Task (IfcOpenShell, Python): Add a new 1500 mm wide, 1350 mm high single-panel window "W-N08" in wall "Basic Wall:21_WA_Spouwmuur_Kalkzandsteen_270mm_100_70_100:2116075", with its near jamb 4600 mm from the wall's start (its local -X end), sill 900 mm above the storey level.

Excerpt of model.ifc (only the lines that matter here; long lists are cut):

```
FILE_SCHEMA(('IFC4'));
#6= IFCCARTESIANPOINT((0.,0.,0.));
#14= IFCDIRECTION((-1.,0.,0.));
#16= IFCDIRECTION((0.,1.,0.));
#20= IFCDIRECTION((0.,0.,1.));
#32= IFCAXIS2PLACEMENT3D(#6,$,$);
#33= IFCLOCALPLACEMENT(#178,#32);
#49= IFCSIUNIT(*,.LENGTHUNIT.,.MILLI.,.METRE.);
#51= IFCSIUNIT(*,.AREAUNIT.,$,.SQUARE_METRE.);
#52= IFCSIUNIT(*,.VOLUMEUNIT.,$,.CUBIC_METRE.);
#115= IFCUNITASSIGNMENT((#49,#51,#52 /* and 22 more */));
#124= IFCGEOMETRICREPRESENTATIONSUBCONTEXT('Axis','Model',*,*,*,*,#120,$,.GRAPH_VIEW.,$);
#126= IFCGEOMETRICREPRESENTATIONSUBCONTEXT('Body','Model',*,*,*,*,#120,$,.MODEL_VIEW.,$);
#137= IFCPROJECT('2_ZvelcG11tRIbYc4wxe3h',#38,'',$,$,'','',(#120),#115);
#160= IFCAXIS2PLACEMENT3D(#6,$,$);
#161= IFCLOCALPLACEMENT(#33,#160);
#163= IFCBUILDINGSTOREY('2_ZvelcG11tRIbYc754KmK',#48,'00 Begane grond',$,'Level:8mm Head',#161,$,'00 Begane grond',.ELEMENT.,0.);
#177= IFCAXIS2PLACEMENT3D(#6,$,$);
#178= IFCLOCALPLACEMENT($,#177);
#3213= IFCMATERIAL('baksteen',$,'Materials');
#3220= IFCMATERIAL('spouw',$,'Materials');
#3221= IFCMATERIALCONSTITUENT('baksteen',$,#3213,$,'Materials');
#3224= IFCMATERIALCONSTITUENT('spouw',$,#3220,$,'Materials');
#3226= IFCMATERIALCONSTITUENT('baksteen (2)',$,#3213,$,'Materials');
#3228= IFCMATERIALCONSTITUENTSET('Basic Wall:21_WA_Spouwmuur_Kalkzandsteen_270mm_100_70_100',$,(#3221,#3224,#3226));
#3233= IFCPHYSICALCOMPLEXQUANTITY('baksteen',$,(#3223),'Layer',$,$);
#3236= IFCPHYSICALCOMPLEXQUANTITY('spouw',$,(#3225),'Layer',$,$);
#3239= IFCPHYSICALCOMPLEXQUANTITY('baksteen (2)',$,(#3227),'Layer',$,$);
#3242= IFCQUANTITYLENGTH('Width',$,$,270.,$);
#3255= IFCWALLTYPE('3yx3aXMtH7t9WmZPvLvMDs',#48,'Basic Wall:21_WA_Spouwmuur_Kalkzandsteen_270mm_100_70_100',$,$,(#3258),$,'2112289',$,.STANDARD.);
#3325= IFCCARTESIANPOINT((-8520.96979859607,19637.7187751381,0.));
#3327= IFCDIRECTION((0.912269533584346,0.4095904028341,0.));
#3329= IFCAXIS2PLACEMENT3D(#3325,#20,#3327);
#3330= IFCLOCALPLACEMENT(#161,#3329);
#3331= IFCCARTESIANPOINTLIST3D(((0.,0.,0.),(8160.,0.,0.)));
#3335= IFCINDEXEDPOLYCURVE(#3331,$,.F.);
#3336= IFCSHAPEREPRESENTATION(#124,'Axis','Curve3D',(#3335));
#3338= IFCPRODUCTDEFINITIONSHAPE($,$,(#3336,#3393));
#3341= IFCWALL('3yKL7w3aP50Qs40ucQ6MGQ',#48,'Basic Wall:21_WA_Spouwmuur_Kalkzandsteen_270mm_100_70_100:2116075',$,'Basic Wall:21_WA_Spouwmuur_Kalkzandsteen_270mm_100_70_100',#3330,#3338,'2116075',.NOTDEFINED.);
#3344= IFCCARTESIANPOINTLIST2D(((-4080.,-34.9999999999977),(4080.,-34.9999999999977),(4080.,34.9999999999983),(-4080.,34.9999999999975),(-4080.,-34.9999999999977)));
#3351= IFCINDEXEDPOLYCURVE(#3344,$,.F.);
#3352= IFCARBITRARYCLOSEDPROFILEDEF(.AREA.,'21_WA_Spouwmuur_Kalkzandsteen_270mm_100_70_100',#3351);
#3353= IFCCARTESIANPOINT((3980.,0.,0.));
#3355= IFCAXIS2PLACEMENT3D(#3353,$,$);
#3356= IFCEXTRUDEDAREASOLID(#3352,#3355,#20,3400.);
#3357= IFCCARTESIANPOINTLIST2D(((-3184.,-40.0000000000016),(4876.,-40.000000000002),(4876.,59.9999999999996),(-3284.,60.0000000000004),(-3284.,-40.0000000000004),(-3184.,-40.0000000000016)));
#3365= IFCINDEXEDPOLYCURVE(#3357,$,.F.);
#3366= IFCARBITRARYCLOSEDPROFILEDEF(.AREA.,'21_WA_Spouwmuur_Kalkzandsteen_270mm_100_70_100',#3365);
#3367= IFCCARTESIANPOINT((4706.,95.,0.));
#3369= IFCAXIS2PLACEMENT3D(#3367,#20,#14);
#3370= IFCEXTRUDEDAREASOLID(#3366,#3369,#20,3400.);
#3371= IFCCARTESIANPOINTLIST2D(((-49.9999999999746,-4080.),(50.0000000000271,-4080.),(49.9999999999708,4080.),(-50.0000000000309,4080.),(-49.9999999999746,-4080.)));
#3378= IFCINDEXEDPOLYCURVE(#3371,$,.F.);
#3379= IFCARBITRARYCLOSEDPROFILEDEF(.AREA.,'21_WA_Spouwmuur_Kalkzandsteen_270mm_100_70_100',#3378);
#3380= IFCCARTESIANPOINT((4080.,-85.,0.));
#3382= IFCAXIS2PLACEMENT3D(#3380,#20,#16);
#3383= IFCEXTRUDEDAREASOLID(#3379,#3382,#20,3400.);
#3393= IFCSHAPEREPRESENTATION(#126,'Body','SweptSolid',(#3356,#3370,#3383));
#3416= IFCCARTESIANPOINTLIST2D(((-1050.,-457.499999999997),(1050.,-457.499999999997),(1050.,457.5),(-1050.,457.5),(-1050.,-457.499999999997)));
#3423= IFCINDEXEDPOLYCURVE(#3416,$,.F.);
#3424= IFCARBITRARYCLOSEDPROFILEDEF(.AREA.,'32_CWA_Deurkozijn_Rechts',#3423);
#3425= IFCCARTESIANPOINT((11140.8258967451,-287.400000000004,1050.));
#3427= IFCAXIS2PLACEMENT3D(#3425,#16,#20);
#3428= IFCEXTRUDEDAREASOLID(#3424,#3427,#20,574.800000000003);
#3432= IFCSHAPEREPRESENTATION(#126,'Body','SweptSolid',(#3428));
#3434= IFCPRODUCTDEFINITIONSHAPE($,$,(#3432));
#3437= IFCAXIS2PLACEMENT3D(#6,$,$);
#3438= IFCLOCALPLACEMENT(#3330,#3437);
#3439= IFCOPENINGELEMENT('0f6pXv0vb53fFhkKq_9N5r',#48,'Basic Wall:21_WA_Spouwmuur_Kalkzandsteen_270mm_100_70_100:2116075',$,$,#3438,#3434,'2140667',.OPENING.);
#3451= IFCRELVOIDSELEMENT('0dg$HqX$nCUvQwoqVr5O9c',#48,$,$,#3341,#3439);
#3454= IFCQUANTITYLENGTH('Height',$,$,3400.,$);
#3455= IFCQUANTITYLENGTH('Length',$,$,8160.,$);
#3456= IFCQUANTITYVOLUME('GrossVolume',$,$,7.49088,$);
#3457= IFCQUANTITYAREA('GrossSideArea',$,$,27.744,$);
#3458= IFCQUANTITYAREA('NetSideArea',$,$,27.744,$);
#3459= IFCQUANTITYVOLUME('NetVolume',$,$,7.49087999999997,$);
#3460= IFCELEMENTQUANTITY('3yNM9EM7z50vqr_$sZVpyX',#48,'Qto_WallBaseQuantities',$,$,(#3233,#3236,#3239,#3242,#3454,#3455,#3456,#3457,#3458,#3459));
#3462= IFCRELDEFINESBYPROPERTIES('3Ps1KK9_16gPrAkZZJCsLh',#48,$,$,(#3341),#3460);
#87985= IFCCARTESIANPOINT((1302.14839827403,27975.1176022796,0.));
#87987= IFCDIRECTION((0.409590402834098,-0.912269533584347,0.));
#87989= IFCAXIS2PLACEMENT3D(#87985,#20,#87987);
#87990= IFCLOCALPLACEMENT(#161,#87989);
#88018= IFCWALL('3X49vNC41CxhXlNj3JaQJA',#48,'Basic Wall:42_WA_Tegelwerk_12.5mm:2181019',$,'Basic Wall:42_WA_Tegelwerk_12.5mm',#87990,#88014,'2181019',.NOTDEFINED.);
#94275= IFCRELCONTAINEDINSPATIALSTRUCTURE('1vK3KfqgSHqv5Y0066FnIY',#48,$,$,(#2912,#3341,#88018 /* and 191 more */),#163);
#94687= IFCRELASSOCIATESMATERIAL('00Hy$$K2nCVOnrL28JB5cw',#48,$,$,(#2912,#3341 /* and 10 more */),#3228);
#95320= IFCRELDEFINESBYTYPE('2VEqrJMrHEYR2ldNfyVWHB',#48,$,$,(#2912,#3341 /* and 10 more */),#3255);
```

```python
import numpy as np
import ifcopenshell
import ifcopenshell.api.feature
import ifcopenshell.api.geometry
import ifcopenshell.api.pset
import ifcopenshell.api.root
import ifcopenshell.api.spatial
import ifcopenshell.geom
import ifcopenshell.util.element
import ifcopenshell.util.placement
import ifcopenshell.util.representation
import ifcopenshell.util.shape
import ifcopenshell.util.unit

model = ifcopenshell.open("model.ifc")
unit_scale = ifcopenshell.util.unit.calculate_unit_scale(model)
area_scale = ifcopenshell.util.unit.calculate_unit_scale(model, "AREAUNIT")
volume_scale = ifcopenshell.util.unit.calculate_unit_scale(model, "VOLUMEUNIT")
settings = ifcopenshell.geom.settings()


def volume(element):
    """Net volume in cubic metres, openings subtracted."""
    shape = ifcopenshell.geom.create_shape(settings, element)
    return ifcopenshell.util.shape.get_volume(shape.geometry)


wall = model.by_guid("3yKL7w3aP50Qs40ucQ6MGQ")
storey = ifcopenshell.util.element.get_container(wall, ifc_class="IfcBuildingStorey")
context = ifcopenshell.util.representation.get_context(model, "Model", "Body", "MODEL_VIEW")
before = volume(wall)

width, height, from_end, sill = 1.5, 1.35, 4.6, 0.9  # metres

# The wall runs along its own X axis, and the end named is its -X end.
wall_shape = ifcopenshell.geom.create_shape(settings, wall)
x, y, z = ifcopenshell.util.shape.get_vertices(wall_shape.geometry).T
start = x.min() + from_end
face, thickness = float(y.min()), float(y.max() - y.min())
wall_matrix = ifcopenshell.util.placement.get_local_placement(wall.ObjectPlacement)
level = ifcopenshell.util.placement.get_local_placement(storey.ObjectPlacement)[2, 3]


def in_wall(x, y):
    """Placement at x, y metres in the wall's axes, at sill height."""
    matrix = wall_matrix.copy()
    matrix[:, 3] = wall_matrix @ np.array([x / unit_scale, y / unit_scale, 0.0, 1.0])
    matrix[2, 3] = level + sill / unit_scale
    return matrix


# Opening: a box that overshoots both wall faces by 50 mm.
opening = ifcopenshell.api.root.create_entity(model, ifc_class="IfcOpeningElement", predefined_type="OPENING")
box = ifcopenshell.api.geometry.add_wall_representation(
    model, context=context, length=width, height=height, thickness=thickness + 0.1
)
ifcopenshell.api.geometry.assign_representation(model, product=opening, representation=box)
ifcopenshell.api.geometry.edit_object_placement(model, product=opening, matrix=in_wall(start, face - 0.05), is_si=False)
ifcopenshell.api.feature.add_feature(model, feature=opening, element=wall)

window = ifcopenshell.api.root.create_entity(model, ifc_class="IfcWindow", name="W-N08", predefined_type="WINDOW")
window.OverallWidth, window.OverallHeight = width / unit_scale, height / unit_scale
window.PartitioningType = "SINGLE_PANEL"
body = ifcopenshell.api.geometry.add_window_representation(
    model,
    context=context,
    overall_width=window.OverallWidth,
    overall_height=window.OverallHeight,
    partition_type="SINGLE_PANEL",
)
ifcopenshell.api.geometry.assign_representation(model, product=window, representation=body)
ifcopenshell.api.spatial.assign_container(model, products=[window], relating_structure=storey)
ifcopenshell.api.feature.add_filling(model, opening=opening, element=window)

# Centre the window in the wall's thickness.
ifcopenshell.api.geometry.edit_object_placement(model, product=window, matrix=in_wall(start, face), is_si=False)
window_shape = ifcopenshell.geom.create_shape(settings, window)
depth = ifcopenshell.util.shape.get_vertices(window_shape.geometry)[:, 1]
offset = face + thickness / 2 - (depth.min() + depth.max()) / 2
ifcopenshell.api.geometry.edit_object_placement(model, product=window, matrix=in_wall(start, offset), is_si=False)

after = volume(wall)

# Update the wall's stored quantities.
qto = model.by_id(ifcopenshell.util.element.get_pset(wall, "Qto_WallBaseQuantities", should_inherit=False)["id"])
ifcopenshell.api.pset.edit_qto(model, qto=qto, properties={
    "NetSideArea": after / thickness / area_scale,
    "NetVolume": after / volume_scale,
})

print(f"wall volume {before:.3f} -> {after:.3f} m3")

model.write("model_updated.ifc")
```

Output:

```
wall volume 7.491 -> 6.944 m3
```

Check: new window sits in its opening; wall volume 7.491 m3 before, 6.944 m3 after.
